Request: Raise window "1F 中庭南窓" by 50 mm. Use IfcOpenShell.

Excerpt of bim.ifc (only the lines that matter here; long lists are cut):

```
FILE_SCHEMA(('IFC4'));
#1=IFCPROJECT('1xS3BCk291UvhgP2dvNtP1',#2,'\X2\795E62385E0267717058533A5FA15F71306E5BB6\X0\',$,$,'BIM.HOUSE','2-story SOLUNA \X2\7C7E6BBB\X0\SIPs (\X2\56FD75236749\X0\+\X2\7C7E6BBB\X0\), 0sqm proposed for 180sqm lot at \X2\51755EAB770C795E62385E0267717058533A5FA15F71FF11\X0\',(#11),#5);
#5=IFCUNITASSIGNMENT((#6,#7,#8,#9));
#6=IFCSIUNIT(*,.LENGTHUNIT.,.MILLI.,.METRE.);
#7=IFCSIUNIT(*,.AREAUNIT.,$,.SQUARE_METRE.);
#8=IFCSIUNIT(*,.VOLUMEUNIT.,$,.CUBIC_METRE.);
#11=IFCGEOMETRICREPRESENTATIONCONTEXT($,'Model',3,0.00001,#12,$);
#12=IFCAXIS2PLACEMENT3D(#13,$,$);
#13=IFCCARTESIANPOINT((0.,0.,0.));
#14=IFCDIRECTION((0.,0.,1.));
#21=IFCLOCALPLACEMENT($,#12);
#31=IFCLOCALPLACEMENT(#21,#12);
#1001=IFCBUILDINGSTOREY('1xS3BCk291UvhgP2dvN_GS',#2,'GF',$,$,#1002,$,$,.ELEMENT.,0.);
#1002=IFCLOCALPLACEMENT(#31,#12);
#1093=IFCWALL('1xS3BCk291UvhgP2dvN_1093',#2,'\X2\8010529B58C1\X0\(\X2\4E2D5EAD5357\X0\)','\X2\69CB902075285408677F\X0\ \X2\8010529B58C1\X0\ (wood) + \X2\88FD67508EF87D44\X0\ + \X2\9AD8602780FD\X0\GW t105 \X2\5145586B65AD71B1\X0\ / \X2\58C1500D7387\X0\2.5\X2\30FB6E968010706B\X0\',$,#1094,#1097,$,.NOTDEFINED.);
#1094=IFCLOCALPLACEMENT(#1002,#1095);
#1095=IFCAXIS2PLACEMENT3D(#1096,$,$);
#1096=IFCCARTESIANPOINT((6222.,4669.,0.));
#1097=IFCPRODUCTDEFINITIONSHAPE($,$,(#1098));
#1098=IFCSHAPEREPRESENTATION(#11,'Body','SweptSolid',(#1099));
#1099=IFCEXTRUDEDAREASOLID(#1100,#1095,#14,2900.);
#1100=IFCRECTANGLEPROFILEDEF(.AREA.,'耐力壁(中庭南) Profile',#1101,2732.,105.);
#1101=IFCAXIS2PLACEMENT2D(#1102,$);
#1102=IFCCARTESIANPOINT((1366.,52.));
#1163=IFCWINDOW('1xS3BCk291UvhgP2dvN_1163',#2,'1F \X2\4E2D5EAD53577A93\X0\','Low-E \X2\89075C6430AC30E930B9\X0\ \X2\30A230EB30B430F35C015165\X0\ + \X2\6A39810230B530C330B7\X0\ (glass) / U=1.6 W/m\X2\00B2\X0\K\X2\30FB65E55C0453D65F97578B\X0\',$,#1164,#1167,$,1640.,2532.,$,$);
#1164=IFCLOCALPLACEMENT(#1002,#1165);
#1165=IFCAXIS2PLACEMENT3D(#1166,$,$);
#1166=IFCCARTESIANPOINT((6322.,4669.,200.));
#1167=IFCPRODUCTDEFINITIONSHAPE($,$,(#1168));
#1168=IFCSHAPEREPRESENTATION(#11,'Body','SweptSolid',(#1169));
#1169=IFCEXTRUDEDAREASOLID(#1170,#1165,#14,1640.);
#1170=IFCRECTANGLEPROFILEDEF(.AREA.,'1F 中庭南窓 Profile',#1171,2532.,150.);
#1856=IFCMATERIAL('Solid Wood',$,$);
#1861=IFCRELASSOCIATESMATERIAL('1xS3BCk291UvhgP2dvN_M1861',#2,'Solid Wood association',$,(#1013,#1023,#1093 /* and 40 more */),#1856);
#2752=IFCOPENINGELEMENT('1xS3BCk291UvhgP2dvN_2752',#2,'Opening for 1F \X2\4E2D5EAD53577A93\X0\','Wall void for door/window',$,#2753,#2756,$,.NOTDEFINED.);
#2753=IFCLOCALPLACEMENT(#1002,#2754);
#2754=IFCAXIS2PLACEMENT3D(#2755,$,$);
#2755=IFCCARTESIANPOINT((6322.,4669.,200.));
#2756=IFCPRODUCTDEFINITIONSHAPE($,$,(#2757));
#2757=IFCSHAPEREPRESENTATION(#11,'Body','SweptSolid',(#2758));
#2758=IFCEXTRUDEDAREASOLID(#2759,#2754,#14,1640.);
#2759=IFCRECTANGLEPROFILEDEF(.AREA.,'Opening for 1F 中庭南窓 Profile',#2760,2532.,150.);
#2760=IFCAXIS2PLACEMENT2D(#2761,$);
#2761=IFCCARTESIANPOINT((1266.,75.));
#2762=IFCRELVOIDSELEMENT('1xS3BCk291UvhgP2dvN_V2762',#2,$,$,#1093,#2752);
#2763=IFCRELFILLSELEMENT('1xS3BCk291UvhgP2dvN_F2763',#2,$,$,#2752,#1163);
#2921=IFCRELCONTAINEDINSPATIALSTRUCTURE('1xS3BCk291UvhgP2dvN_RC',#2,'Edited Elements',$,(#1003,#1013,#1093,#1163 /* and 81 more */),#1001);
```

```python
import numpy as np
import ifcopenshell
import ifcopenshell.api.geometry
import ifcopenshell.util.placement
import ifcopenshell.util.unit

model = ifcopenshell.open("bim.ifc")
unit_scale = ifcopenshell.util.unit.calculate_unit_scale(model)

window = model.by_guid("1xS3BCk291UvhgP2dvN_1163")
opening = window.FillsVoids[0].RelatingOpeningElement
dz = 50.0

shift = np.array([0.0, 0.0, dz])
# The window is not placed relative to its opening, so move both.
for product in (opening, window):
    matrix = ifcopenshell.util.placement.get_local_placement(product.ObjectPlacement)
    matrix[:3, 3] += shift
    ifcopenshell.api.geometry.edit_object_placement(model, product=product, matrix=matrix, is_si=False)

print(f"moved by {dz * unit_scale:+.3f} m")

model.write("bim_updated.ifc")
```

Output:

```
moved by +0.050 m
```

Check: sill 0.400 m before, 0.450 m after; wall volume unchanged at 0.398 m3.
